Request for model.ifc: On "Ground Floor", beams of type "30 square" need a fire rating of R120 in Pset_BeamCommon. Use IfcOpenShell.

First a look at what the model holds.

```python
import ifcopenshell
import ifcopenshell.util.element

model = ifcopenshell.open("model.ifc")
print(model.schema)
storey = next(s for s in model.by_type("IfcBuildingStorey") if s.Name == "Ground Floor")
beams = [e for e in ifcopenshell.util.element.get_decomposition(storey) if e.is_a("IfcBeam")]
seen = {}
for e in beams:
    element_type = ifcopenshell.util.element.get_type(e)
    key = (element_type.Name if element_type != e and element_type else None, ifcopenshell.util.element.get_pset(e, "Pset_BeamCommon", "FireRating"))
    seen[key] = seen.get(key, 0) + 1
for (name, value), count in sorted(seen.items(), key=str):
    print(count, "x", name, "|", value)
```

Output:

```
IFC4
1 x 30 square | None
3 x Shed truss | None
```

```python
import ifcopenshell
import ifcopenshell.api.pset
import ifcopenshell.util.element

model = ifcopenshell.open("model.ifc")

storey = next(s for s in model.by_type("IfcBuildingStorey") if s.Name == "Ground Floor")
beams = [e for e in ifcopenshell.util.element.get_decomposition(storey) if e.is_a("IfcBeam")]

count = 0
for e in beams:
    element_type = ifcopenshell.util.element.get_type(e)
    if element_type in (None, e) or element_type.Name != "30 square":
        continue
    # add_pset returns the element's existing set when there is one.
    pset = ifcopenshell.api.pset.add_pset(model, product=e, name="Pset_BeamCommon")
    ifcopenshell.api.pset.edit_pset(model, pset=pset, properties={"FireRating": "R120"})
    count += 1

print(count, "beams updated")

model.write("model_updated.ifc")
```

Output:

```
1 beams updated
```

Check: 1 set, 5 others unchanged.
